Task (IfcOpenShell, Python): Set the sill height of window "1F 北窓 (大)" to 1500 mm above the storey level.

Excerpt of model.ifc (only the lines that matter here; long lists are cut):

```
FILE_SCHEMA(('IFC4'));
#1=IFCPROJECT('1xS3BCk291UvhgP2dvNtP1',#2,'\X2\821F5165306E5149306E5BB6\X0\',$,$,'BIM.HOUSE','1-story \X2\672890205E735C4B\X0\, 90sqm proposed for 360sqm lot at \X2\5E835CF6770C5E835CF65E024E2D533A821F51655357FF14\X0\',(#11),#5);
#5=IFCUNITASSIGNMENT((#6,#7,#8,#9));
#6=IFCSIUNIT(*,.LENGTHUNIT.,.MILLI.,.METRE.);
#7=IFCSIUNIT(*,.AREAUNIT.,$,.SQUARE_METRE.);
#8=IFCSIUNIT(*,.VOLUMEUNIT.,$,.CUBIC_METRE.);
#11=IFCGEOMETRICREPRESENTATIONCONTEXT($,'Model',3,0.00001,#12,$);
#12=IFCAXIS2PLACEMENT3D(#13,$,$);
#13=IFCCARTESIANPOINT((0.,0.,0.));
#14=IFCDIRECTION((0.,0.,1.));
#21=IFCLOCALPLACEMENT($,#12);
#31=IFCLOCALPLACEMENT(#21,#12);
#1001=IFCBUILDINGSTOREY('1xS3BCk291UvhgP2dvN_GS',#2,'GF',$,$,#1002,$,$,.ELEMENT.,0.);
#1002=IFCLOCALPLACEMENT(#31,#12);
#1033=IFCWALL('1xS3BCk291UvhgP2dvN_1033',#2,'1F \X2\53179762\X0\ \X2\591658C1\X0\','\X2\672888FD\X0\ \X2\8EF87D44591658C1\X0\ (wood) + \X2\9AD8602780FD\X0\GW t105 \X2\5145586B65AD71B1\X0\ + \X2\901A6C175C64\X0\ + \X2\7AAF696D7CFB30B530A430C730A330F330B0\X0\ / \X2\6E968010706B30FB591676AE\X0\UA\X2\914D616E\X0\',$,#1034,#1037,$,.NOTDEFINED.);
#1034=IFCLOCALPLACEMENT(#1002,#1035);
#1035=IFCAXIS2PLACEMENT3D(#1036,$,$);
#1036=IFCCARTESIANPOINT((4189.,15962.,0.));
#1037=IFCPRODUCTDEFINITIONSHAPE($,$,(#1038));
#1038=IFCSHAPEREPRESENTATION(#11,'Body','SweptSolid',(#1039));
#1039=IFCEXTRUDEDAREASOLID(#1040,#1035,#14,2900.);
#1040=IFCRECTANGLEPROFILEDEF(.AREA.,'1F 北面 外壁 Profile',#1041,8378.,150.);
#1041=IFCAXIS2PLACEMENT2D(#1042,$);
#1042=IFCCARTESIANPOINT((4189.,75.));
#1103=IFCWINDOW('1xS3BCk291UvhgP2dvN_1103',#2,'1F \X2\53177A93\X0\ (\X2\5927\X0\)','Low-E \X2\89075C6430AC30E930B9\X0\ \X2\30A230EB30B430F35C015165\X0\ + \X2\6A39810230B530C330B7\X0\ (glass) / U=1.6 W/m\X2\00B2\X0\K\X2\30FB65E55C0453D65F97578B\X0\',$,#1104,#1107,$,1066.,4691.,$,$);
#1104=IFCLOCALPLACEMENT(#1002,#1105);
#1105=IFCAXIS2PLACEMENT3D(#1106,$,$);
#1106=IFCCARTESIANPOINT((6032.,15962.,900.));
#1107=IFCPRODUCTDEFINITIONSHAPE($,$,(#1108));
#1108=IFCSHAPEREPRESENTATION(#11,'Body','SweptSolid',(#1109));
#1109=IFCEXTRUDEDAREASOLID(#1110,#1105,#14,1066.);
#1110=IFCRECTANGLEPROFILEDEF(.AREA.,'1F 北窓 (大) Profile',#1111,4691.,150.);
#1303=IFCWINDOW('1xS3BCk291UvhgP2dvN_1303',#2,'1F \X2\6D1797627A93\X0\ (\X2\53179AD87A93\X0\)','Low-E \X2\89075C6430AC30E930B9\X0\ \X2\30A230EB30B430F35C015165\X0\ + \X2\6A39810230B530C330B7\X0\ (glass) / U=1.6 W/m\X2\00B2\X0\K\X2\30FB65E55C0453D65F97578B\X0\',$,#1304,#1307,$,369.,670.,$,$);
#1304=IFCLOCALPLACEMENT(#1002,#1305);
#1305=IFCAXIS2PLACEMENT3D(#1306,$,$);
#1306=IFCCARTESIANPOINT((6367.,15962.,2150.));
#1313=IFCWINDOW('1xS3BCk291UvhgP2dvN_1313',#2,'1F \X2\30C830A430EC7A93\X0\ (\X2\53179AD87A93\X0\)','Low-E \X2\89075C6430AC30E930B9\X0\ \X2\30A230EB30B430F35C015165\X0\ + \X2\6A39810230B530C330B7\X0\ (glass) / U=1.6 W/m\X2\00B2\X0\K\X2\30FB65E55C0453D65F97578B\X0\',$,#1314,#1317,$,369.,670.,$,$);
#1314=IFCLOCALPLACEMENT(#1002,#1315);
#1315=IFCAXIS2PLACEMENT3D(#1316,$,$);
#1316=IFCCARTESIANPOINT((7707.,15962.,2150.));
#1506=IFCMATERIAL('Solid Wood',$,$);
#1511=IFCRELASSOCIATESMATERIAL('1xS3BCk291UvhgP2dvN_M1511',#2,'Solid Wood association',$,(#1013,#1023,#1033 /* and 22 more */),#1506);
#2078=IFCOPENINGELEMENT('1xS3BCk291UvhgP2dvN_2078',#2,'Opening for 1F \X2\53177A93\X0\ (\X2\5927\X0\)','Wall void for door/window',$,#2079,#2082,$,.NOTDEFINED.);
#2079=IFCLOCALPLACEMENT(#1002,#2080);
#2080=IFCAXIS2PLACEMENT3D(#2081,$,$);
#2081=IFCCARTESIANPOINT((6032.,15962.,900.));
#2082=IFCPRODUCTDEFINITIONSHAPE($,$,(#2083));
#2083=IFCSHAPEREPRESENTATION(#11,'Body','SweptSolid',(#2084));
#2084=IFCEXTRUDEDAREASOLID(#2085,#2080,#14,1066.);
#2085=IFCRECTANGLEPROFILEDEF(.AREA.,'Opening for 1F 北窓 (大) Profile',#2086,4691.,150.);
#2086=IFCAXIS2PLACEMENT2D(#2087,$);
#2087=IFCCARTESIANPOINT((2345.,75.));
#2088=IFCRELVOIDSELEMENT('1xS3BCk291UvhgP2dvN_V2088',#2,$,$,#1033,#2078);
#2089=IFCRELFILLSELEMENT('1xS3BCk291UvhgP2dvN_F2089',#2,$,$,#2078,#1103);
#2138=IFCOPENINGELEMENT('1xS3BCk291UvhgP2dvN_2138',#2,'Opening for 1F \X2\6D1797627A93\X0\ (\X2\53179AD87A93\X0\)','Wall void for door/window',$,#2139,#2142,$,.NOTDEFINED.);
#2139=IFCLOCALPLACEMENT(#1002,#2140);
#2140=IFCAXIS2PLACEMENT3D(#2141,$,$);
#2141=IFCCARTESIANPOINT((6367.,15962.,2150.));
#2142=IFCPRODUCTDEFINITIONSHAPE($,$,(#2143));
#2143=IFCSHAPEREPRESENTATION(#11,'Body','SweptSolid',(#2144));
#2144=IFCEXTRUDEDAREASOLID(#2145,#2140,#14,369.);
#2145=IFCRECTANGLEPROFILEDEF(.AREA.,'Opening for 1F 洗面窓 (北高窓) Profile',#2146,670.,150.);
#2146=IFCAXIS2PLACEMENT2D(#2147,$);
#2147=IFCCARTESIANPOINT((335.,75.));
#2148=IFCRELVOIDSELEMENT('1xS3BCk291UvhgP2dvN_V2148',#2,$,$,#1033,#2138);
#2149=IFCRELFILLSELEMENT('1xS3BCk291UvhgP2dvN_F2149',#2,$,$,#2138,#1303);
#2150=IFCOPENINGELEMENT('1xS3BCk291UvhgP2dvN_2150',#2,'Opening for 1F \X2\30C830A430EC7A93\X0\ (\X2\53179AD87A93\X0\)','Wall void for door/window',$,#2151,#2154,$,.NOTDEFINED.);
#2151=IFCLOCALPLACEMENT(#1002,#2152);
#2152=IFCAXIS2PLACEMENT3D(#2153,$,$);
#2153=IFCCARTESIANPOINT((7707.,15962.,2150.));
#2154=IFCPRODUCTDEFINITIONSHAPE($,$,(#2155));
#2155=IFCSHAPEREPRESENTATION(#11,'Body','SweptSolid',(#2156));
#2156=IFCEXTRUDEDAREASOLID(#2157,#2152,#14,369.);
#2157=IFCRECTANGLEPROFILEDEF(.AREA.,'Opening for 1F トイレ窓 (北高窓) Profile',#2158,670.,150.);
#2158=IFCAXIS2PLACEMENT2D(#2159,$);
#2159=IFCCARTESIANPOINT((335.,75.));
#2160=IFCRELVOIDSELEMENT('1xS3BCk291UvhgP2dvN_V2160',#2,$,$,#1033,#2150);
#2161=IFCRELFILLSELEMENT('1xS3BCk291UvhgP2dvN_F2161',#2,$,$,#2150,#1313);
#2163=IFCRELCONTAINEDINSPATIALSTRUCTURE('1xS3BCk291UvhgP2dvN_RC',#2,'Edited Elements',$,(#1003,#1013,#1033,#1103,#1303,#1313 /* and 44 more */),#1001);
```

```python
import numpy as np
import ifcopenshell
import ifcopenshell.api.geometry
import ifcopenshell.geom
import ifcopenshell.util.element
import ifcopenshell.util.placement
import ifcopenshell.util.shape
import ifcopenshell.util.unit

model = ifcopenshell.open("model.ifc")
unit_scale = ifcopenshell.util.unit.calculate_unit_scale(model)

window = model.by_guid("1xS3BCk291UvhgP2dvN_1103")
opening = window.FillsVoids[0].RelatingOpeningElement
storey = ifcopenshell.util.element.get_container(window, ifc_class="IfcBuildingStorey")
level = ifcopenshell.util.placement.get_local_placement(storey.ObjectPlacement)[2, 3]

# The opening's origin need not be at the sill, so measure its lowest point.
shape = ifcopenshell.geom.create_shape(ifcopenshell.geom.settings(), opening)
bottom = ifcopenshell.util.shape.get_shape_bottom_elevation(shape, shape.geometry) / unit_scale
dz = level + 1500.0 - bottom

shift = np.array([0.0, 0.0, dz])
# The window is not placed relative to its opening, so move both.
for product in (opening, window):
    matrix = ifcopenshell.util.placement.get_local_placement(product.ObjectPlacement)
    matrix[:3, 3] += shift
    ifcopenshell.api.geometry.edit_object_placement(model, product=product, matrix=matrix, is_si=False)

print(f"moved by {dz * unit_scale:+.3f} m")

model.write("model_v2.ifc")
```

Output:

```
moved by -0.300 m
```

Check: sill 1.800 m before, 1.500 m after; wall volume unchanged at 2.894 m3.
